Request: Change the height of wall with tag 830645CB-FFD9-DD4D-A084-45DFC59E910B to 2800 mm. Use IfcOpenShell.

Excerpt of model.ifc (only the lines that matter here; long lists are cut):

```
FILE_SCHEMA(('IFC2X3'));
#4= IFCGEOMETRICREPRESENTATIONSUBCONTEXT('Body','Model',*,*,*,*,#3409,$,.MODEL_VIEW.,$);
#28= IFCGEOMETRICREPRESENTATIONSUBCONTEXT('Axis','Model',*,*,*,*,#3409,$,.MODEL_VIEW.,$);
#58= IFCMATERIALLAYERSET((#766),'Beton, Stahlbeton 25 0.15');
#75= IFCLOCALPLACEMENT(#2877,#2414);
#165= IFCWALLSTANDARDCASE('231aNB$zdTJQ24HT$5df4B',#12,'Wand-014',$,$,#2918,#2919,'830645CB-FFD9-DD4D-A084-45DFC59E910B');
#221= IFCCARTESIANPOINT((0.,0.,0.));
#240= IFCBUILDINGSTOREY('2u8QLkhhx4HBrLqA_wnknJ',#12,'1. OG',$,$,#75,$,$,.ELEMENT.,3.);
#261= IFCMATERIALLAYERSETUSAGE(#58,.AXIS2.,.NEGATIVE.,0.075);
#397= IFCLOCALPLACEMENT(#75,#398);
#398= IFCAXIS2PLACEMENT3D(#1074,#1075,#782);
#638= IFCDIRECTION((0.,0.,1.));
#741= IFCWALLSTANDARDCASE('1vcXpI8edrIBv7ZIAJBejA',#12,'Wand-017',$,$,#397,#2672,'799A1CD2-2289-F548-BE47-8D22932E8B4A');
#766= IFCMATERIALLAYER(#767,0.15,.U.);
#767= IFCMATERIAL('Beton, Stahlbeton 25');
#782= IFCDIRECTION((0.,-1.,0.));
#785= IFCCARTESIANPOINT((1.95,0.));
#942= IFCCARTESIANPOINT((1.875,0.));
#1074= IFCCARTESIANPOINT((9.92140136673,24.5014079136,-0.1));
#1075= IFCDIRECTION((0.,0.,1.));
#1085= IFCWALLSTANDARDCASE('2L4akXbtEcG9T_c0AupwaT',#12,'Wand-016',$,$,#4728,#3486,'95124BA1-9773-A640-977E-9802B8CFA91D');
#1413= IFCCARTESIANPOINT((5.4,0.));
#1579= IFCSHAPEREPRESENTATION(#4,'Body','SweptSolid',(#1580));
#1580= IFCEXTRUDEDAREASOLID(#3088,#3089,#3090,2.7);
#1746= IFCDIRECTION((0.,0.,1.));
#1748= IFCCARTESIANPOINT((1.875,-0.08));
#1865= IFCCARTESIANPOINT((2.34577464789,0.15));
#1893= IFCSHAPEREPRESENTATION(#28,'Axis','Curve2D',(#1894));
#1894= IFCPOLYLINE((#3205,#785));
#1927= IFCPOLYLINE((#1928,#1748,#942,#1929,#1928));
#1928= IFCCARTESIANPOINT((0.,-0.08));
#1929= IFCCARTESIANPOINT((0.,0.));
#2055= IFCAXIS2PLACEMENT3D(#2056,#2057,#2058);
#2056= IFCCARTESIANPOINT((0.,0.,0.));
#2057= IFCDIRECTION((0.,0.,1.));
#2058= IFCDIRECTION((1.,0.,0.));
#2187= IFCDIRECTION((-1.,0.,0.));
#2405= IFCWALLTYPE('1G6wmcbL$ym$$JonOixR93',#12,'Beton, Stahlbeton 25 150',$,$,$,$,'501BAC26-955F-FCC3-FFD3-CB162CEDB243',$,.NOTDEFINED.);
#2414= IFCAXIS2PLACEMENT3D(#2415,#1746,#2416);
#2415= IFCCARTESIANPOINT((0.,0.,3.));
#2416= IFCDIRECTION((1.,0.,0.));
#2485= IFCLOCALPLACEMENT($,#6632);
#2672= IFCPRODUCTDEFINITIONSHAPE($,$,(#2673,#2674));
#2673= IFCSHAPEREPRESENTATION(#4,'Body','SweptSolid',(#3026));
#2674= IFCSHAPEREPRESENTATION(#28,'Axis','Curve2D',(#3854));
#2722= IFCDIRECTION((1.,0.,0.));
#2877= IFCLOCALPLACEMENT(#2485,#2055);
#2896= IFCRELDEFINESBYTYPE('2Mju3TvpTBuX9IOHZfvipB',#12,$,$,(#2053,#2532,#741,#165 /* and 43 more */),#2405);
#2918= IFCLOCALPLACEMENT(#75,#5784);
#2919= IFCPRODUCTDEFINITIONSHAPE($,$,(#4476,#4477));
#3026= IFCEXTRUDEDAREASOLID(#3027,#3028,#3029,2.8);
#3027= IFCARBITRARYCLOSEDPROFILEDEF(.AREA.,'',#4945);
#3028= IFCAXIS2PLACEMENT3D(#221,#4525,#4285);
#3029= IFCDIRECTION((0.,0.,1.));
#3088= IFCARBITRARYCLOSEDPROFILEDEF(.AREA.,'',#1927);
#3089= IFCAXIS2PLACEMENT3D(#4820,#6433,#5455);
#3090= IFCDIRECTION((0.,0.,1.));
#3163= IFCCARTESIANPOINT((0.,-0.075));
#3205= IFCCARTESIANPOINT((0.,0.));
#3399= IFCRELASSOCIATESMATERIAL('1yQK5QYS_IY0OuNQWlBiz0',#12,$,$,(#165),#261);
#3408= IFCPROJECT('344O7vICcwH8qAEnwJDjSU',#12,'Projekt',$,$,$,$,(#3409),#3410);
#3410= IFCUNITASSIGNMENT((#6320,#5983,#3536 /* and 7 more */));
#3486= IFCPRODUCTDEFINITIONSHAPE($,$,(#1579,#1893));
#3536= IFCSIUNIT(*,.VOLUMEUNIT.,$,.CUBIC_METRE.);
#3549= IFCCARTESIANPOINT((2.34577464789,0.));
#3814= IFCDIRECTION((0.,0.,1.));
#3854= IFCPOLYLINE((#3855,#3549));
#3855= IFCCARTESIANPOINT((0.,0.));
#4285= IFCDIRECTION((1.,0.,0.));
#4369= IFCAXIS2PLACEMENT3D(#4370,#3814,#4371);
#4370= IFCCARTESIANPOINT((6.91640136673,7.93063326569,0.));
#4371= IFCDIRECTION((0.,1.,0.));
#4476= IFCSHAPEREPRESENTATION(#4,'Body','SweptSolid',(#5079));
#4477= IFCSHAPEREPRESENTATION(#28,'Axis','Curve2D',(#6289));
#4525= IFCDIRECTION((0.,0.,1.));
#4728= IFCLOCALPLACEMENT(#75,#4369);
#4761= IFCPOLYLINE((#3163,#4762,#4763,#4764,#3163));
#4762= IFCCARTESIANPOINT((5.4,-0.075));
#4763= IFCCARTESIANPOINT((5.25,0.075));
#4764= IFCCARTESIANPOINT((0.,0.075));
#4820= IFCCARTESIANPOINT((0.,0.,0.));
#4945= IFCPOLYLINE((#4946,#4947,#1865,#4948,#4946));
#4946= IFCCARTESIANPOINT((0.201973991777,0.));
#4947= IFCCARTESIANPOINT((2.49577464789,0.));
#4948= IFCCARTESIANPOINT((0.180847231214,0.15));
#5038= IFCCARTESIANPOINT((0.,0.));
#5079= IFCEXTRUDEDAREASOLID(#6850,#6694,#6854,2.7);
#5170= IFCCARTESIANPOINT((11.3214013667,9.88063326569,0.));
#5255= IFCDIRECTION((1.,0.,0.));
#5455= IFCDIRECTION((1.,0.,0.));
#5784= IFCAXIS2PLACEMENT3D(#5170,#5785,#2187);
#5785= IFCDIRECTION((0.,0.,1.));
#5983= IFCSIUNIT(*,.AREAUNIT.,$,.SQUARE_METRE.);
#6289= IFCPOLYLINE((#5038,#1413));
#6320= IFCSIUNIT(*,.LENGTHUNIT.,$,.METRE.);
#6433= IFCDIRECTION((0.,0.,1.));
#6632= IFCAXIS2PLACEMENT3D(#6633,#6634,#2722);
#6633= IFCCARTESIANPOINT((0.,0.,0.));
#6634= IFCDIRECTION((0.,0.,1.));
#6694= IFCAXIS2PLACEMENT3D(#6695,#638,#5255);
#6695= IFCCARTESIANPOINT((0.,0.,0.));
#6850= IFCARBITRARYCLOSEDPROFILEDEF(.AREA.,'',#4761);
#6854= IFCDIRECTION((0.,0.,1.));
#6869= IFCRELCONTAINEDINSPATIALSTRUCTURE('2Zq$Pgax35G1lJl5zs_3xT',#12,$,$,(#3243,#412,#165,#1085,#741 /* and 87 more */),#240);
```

```python
import ifcopenshell
import ifcopenshell.geom
import ifcopenshell.util.representation
import ifcopenshell.util.shape

model = ifcopenshell.open("model.ifc")
settings = ifcopenshell.geom.settings()


def volume(element):
    """Net volume in cubic metres, openings subtracted."""
    shape = ifcopenshell.geom.create_shape(settings, element)
    return ifcopenshell.util.shape.get_volume(shape.geometry)


wall = model.by_guid("231aNB$zdTJQ24HT$5df4B")
before = volume(wall)

body = ifcopenshell.util.representation.get_representation(wall, "Model", "Body")
solid = body.Items[0]
old_height = solid.Depth
solid.Depth = 2.8
after = volume(wall)

print(f"height {old_height:g} -> {solid.Depth:g}, volume {before:.3f} -> {after:.3f} m3")

model.write("model-out.ifc")
```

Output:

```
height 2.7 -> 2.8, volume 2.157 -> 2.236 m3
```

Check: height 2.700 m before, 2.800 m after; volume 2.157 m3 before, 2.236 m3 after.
